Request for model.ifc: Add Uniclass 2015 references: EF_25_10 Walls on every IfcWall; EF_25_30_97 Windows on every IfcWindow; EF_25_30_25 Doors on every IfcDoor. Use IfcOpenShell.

First a look at what the model holds.

```python
import ifcopenshell

model = ifcopenshell.open("model.ifc")
print(model.schema)
print("classifications:", [c.Name for c in model.by_type("IfcClassification")])
for ifc_class in ("IfcDoor", "IfcRoof", "IfcStair", "IfcWall", "IfcWindow"):
    print(ifc_class, len(model.by_type(ifc_class)))
```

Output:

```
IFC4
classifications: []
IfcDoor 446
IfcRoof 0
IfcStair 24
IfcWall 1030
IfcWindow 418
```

```python
import ifcopenshell
import ifcopenshell.api.classification

model = ifcopenshell.open("model.ifc")

system = ifcopenshell.api.classification.add_classification(model, classification="Uniclass 2015")

codes = {
    "IfcWall": ("EF_25_10", "Walls"),
    "IfcWindow": ("EF_25_30_97", "Windows"),
    "IfcDoor": ("EF_25_30_25", "Doors"),
}
for ifc_class, (code, name) in codes.items():
    products = model.by_type(ifc_class)
    ifcopenshell.api.classification.add_reference(
        model, products=products, classification=system, identification=code, name=name
    )
    print(code, len(products))

model.write("model_updated.ifc")
```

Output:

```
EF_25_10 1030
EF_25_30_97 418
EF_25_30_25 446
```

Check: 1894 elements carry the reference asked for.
